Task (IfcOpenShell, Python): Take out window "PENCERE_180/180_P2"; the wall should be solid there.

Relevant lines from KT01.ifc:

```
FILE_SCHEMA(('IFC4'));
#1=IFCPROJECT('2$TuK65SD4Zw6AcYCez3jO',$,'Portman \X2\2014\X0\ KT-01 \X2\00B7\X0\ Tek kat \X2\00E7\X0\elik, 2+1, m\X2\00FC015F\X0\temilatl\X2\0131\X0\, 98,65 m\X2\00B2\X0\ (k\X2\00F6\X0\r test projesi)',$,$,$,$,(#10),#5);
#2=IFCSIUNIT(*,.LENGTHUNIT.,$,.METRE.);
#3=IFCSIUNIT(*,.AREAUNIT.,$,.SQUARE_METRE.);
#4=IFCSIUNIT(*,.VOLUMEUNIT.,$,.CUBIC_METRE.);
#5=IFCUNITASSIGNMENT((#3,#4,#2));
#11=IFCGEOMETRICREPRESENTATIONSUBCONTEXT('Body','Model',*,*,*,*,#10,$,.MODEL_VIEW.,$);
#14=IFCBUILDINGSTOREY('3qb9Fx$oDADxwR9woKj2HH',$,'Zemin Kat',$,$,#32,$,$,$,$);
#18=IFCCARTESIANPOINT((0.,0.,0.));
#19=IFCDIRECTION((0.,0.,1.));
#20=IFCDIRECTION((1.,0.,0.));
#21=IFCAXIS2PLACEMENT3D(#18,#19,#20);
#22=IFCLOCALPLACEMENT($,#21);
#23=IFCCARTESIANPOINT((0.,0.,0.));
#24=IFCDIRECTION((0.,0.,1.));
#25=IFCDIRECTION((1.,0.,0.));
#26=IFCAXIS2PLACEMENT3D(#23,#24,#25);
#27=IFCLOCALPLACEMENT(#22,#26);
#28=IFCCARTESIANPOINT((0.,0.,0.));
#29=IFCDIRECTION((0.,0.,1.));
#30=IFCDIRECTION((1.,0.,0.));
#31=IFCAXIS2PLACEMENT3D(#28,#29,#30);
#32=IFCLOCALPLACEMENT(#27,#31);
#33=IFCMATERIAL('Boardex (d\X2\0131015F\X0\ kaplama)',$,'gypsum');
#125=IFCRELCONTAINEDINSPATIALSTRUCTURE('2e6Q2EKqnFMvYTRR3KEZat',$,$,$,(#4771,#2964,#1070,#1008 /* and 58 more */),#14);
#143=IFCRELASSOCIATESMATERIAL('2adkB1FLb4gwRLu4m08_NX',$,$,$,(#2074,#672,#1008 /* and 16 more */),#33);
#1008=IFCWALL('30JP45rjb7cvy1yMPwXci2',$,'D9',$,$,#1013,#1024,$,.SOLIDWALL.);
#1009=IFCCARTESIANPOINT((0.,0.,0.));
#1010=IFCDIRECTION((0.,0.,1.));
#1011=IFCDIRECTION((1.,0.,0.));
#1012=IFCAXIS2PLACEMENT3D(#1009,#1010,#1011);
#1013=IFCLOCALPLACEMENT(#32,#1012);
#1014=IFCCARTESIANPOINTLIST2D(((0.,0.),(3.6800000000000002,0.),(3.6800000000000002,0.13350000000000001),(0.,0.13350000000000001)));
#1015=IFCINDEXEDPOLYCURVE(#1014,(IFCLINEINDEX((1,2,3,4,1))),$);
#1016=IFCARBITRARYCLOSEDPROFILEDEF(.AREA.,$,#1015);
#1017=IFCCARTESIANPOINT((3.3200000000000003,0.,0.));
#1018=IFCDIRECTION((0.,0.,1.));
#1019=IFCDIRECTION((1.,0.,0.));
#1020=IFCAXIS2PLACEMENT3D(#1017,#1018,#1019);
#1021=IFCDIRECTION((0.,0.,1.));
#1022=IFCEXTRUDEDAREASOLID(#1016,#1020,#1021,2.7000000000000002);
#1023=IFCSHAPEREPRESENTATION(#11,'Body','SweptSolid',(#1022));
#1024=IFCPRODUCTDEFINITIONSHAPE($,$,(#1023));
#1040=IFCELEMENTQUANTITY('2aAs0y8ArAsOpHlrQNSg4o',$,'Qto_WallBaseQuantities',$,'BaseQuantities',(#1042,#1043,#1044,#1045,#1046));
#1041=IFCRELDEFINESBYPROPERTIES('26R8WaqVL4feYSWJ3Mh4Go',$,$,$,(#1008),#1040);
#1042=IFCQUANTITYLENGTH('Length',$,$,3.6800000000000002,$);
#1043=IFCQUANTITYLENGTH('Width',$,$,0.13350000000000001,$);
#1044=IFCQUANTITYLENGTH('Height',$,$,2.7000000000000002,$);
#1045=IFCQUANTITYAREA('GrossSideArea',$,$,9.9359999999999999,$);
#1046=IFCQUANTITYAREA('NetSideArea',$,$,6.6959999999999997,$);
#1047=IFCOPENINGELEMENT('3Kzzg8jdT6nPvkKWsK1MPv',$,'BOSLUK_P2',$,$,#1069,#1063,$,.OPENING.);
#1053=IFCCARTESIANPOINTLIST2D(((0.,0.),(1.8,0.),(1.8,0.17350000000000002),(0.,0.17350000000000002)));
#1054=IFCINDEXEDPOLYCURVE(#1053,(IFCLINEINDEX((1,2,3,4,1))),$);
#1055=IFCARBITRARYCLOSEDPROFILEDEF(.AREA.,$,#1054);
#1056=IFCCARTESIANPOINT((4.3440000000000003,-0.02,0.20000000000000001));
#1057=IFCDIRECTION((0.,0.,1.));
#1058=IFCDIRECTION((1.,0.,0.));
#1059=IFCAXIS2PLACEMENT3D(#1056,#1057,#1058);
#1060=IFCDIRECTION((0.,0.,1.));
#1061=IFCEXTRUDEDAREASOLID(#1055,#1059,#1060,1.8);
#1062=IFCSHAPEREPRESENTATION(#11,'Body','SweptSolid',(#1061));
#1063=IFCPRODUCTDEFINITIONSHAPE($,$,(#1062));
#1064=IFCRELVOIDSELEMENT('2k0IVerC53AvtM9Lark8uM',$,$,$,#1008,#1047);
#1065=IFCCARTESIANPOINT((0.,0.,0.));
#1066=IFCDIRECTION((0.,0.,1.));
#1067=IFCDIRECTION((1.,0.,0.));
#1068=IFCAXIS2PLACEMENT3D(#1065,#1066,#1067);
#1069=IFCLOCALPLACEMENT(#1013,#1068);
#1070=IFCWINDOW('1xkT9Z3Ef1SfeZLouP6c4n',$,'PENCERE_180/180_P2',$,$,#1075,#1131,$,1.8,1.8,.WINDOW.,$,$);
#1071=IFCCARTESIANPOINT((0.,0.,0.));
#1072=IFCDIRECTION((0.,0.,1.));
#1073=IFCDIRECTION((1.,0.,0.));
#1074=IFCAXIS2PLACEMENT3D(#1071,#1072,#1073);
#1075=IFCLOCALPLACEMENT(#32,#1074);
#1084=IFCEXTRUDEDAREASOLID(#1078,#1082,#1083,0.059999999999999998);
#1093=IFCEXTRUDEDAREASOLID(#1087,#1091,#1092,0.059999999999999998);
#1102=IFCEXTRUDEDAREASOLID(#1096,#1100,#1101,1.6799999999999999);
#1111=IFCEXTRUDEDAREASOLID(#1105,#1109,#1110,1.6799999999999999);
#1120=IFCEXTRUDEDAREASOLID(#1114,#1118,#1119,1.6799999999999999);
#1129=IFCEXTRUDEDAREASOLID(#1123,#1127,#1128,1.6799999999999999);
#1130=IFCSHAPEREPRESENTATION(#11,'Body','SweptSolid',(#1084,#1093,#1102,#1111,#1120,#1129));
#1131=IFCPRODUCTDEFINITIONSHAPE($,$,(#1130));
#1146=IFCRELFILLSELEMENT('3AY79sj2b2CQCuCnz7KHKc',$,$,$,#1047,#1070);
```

```python
import ifcopenshell
import ifcopenshell.api.feature
import ifcopenshell.api.pset
import ifcopenshell.api.root
import ifcopenshell.geom
import ifcopenshell.util.element
import ifcopenshell.util.shape
import ifcopenshell.util.unit

model = ifcopenshell.open("KT01.ifc")
area_scale = ifcopenshell.util.unit.calculate_unit_scale(model, "AREAUNIT")
settings = ifcopenshell.geom.settings()


def volume(element):
    """Net volume in cubic metres, openings subtracted."""
    shape = ifcopenshell.geom.create_shape(settings, element)
    return ifcopenshell.util.shape.get_volume(shape.geometry)


window = model.by_guid("1xkT9Z3Ef1SfeZLouP6c4n")
opening = window.FillsVoids[0].RelatingOpeningElement
wall = opening.VoidsElements[0].RelatingBuildingElement
before = volume(wall)

ifcopenshell.api.root.remove_product(model, product=window)
ifcopenshell.api.feature.remove_feature(model, feature=opening)

after = volume(wall)
thickness = 0.1335  # wall thickness in metres

# Update the wall's stored quantities.
qto = model.by_id(ifcopenshell.util.element.get_pset(wall, "Qto_WallBaseQuantities", should_inherit=False)["id"])
ifcopenshell.api.pset.edit_qto(model, qto=qto, properties={"NetSideArea": after / thickness / area_scale})

print(f"wall volume {before:.3f} -> {after:.3f} m3")

model.write("KT01_rev.ifc")
```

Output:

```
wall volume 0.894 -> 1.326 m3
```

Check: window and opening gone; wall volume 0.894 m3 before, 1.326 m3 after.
